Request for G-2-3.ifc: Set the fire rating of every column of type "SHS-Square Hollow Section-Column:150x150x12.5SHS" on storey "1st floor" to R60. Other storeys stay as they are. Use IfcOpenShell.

First a look at what the model holds.

```python
import ifcopenshell
import ifcopenshell.util.element

model = ifcopenshell.open("G-2-3.ifc")
print(model.schema)
storey = next(s for s in model.by_type("IfcBuildingStorey") if s.Name == "1st floor")
columns = [e for e in ifcopenshell.util.element.get_decomposition(storey) if e.is_a("IfcColumn")]
seen = {}
for e in columns:
    element_type = ifcopenshell.util.element.get_type(e)
    key = (element_type.Name if element_type != e and element_type else None, ifcopenshell.util.element.get_pset(e, "Pset_ColumnCommon", "FireRating"))
    seen[key] = seen.get(key, 0) + 1
for (name, value), count in sorted(seen.items(), key=str):
    print(count, "x", name, "|", value)
```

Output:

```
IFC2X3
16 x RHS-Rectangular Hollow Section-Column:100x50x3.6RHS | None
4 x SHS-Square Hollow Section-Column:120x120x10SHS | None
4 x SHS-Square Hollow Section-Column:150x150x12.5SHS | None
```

```python
import ifcopenshell
import ifcopenshell.api.pset
import ifcopenshell.util.element

model = ifcopenshell.open("G-2-3.ifc")

storey = next(s for s in model.by_type("IfcBuildingStorey") if s.Name == "1st floor")
columns = [e for e in ifcopenshell.util.element.get_decomposition(storey) if e.is_a("IfcColumn")]

count = 0
for e in columns:
    element_type = ifcopenshell.util.element.get_type(e)
    if element_type in (None, e) or element_type.Name != "SHS-Square Hollow Section-Column:150x150x12.5SHS":
        continue
    # add_pset returns the element's existing set when there is one.
    pset = ifcopenshell.api.pset.add_pset(model, product=e, name="Pset_ColumnCommon")
    ifcopenshell.api.pset.edit_pset(model, pset=pset, properties={"FireRating": "R60"})
    count += 1

print(count, "columns updated")

model.write("G-2-3_edited.ifc")
```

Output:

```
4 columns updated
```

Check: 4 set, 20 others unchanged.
